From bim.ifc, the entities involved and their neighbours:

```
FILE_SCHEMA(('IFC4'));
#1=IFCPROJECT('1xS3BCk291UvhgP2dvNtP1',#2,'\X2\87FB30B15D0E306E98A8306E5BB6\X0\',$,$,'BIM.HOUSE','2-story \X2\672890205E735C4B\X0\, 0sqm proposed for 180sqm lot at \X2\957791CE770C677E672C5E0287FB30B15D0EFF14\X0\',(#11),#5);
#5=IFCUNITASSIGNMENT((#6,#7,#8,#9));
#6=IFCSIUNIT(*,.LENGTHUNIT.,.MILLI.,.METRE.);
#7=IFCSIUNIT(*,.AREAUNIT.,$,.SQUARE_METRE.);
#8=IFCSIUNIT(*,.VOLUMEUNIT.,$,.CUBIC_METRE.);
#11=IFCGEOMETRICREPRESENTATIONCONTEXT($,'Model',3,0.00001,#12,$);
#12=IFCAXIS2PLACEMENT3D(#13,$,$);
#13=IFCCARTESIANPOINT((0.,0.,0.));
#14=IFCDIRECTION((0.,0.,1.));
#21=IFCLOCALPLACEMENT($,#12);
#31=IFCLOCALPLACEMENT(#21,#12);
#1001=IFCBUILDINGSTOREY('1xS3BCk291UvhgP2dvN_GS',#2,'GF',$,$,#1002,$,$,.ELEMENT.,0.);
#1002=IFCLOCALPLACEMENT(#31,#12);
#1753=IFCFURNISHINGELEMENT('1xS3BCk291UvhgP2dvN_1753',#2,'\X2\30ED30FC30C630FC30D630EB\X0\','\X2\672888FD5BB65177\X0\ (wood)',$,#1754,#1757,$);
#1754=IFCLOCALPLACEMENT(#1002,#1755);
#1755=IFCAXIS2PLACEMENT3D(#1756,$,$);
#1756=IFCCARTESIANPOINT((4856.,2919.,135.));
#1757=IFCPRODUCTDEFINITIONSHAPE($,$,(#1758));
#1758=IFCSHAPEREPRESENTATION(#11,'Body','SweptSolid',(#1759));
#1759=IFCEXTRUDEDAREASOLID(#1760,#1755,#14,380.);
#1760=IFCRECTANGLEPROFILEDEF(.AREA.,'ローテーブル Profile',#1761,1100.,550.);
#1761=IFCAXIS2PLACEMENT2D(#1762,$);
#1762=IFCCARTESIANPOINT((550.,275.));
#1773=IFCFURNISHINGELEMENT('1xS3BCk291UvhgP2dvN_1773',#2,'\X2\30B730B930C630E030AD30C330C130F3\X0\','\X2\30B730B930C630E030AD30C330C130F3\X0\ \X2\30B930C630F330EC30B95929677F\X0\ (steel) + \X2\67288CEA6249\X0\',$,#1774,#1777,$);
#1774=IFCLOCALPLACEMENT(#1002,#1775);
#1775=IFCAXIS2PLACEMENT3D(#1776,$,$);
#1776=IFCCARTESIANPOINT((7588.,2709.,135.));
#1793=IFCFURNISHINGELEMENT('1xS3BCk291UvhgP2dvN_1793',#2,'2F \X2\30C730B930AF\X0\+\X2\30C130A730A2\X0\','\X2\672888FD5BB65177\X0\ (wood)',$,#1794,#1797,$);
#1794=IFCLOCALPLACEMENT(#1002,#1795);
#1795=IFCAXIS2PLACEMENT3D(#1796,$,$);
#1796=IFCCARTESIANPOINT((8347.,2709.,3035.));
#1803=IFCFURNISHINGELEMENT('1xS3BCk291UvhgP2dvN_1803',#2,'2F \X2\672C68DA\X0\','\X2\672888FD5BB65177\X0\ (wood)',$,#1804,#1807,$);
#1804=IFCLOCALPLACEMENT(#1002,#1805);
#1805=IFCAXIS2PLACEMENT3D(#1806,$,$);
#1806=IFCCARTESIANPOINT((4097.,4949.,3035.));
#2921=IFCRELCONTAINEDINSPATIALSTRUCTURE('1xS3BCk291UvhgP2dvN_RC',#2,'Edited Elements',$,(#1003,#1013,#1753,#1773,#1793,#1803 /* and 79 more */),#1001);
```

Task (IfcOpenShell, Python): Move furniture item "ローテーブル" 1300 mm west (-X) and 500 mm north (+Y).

```python
import ifcopenshell
import ifcopenshell.api.geometry
import ifcopenshell.util.placement

model = ifcopenshell.open("bim.ifc")

item = model.by_id(1753)
matrix = ifcopenshell.util.placement.get_local_placement(item.ObjectPlacement)
matrix[0, 3] -= 1300.0
matrix[1, 3] += 500.0
ifcopenshell.api.geometry.edit_object_placement(model, product=item, matrix=matrix, is_si=False)

print(ifcopenshell.util.placement.get_local_placement(item.ObjectPlacement).round(3) + 0.0)

model.write("bim_v2.ifc")
```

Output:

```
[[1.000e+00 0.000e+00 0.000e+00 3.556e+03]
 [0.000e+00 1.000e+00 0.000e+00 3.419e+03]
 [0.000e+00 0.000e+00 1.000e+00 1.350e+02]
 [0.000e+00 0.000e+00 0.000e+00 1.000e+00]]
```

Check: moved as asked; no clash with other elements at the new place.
